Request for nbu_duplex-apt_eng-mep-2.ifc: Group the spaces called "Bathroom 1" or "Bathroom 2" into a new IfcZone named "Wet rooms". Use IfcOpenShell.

First a look at what the model holds.

```python
import ifcopenshell

model = ifcopenshell.open("nbu_duplex-apt_eng-mep-2.ifc")
print(model.schema)
seen = {}
for space in model.by_type("IfcSpace"):
    seen[space.LongName] = seen.get(space.LongName, 0) + 1
for name, count in sorted(seen.items(), key=str):
    print(count, "x", name)
print("zones:", [z.Name for z in model.by_type("IfcZone")][:20])
```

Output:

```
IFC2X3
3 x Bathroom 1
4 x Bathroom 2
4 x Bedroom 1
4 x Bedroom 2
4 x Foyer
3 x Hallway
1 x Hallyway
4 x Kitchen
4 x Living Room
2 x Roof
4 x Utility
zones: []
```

```python
import ifcopenshell
import ifcopenshell.api.group
import ifcopenshell.api.root

model = ifcopenshell.open("nbu_duplex-apt_eng-mep-2.ifc")

names = {"Bathroom 1", "Bathroom 2"}
spaces = [s for s in model.by_type("IfcSpace") if s.LongName in names]

zone = ifcopenshell.api.root.create_entity(model, ifc_class="IfcZone", name="Wet rooms")
ifcopenshell.api.group.assign_group(model, products=spaces, group=zone)
print(len(spaces), "spaces in", zone.Name)

model.write("nbu_duplex-apt_eng-mep-2_updated.ifc")
```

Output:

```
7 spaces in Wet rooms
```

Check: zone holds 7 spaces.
